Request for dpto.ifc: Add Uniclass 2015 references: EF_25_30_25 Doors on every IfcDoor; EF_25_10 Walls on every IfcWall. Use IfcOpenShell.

First a look at what the model holds.

```python
import ifcopenshell

model = ifcopenshell.open("dpto.ifc")
print(model.schema)
print("classifications:", [c.Name for c in model.by_type("IfcClassification")])
for ifc_class in ("IfcDoor", "IfcRoof", "IfcStair", "IfcWall", "IfcWindow"):
    print(ifc_class, len(model.by_type(ifc_class)))
```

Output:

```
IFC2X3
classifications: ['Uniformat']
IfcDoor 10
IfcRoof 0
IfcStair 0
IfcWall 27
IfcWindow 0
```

```python
import ifcopenshell
import ifcopenshell.api.classification

model = ifcopenshell.open("dpto.ifc")

# IFC2X3 requires Source and Edition and has no link from the project to the system.
system = model.create_entity("IfcClassification", Source="NBS", Edition="2015", Name="Uniclass 2015")

codes = {
    "IfcDoor": ("EF_25_30_25", "Doors"),
    "IfcWall": ("EF_25_10", "Walls"),
}
for ifc_class, (code, name) in codes.items():
    products = model.by_type(ifc_class)
    ifcopenshell.api.classification.add_reference(
        model, products=products, classification=system, identification=code, name=name
    )
    print(code, len(products))

model.write("dpto-out.ifc")
```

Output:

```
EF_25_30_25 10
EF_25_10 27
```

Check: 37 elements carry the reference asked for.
